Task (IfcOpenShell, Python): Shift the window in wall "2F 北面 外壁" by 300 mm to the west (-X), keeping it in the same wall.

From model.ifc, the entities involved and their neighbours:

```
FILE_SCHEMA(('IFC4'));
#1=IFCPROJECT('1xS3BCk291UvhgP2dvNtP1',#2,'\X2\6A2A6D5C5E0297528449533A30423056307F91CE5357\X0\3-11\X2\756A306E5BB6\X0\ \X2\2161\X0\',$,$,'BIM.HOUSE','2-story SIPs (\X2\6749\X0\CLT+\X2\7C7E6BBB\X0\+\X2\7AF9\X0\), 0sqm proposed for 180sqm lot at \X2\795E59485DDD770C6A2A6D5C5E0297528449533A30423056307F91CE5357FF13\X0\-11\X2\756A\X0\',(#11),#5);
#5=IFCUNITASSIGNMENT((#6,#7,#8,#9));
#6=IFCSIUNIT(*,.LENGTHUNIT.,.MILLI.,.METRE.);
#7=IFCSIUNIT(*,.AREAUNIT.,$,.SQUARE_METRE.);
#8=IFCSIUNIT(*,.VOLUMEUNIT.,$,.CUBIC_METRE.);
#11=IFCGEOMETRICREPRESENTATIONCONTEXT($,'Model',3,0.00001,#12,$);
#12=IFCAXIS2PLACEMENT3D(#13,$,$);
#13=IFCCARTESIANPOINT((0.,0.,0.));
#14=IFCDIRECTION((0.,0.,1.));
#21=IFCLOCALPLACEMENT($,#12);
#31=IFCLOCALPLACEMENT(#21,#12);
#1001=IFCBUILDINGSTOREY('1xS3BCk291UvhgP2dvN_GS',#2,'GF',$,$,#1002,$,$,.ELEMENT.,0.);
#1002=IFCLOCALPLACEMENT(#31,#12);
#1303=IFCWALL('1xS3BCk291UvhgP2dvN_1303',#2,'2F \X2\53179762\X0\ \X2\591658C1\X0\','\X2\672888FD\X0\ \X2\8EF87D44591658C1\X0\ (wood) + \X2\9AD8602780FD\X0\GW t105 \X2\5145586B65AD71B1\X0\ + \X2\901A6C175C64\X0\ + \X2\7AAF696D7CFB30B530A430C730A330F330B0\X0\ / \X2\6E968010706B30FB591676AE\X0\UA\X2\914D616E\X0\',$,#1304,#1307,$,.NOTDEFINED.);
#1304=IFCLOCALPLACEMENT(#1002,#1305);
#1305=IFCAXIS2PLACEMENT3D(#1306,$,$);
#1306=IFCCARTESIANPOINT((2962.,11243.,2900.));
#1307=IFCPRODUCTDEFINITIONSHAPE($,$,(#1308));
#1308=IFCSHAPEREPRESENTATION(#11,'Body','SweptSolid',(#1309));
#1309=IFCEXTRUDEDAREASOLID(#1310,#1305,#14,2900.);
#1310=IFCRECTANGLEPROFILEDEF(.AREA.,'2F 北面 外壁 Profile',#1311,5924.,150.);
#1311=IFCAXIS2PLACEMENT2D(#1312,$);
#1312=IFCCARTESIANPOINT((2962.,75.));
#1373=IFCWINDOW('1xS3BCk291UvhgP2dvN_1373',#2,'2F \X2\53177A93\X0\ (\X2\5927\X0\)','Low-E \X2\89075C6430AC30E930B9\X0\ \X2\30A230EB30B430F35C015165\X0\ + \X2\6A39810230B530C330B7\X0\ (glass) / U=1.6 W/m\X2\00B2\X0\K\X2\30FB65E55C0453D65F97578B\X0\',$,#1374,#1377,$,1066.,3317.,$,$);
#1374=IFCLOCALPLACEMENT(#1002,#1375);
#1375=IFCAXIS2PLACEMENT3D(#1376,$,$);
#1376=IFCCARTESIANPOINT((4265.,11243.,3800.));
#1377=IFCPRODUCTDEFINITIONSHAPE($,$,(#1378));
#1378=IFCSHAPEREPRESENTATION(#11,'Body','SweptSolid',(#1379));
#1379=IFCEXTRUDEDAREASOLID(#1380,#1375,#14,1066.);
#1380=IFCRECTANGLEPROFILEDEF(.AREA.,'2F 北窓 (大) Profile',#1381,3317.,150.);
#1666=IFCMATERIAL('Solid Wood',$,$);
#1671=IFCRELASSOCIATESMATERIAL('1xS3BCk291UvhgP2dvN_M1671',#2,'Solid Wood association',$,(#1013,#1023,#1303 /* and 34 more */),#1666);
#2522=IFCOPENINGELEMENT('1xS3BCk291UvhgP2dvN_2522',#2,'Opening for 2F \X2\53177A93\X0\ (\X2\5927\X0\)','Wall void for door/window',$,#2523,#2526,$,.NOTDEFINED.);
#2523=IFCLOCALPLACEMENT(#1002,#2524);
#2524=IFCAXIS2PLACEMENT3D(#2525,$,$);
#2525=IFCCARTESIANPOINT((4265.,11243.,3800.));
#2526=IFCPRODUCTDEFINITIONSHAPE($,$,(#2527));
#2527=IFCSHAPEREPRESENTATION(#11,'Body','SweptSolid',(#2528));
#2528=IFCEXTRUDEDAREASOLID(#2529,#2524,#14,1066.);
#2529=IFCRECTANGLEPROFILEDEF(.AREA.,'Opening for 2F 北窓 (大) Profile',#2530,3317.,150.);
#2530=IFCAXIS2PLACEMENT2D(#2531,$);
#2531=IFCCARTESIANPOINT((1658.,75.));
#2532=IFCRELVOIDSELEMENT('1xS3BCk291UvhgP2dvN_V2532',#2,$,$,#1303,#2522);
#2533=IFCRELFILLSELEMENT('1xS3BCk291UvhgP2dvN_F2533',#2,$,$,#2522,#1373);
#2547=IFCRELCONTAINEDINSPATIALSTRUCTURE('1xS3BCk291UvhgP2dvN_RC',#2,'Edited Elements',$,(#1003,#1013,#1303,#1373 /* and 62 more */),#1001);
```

```python
import ifcopenshell
import ifcopenshell.api.geometry
import ifcopenshell.util.placement

model = ifcopenshell.open("model.ifc")

window = model.by_guid("1xS3BCk291UvhgP2dvN_1373")
opening = window.FillsVoids[0].RelatingOpeningElement
wall = opening.VoidsElements[0].RelatingBuildingElement

wall_matrix = ifcopenshell.util.placement.get_local_placement(wall.ObjectPlacement)
shift = wall_matrix[:3, 0] * -300.0
before = ifcopenshell.util.placement.get_local_placement(window.ObjectPlacement)[:3, 3].copy()

# The window is not placed relative to its opening, so move both.
for product in (opening, window):
    matrix = ifcopenshell.util.placement.get_local_placement(product.ObjectPlacement)
    matrix[:3, 3] += shift
    ifcopenshell.api.geometry.edit_object_placement(model, product=product, matrix=matrix, is_si=False)

after = ifcopenshell.util.placement.get_local_placement(window.ObjectPlacement)[:3, 3]
print("window moved by", (after - before).round(3) + 0.0)

model.write("model_rev.ifc")
```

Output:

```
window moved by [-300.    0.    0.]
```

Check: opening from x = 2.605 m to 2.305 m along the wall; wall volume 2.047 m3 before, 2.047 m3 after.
